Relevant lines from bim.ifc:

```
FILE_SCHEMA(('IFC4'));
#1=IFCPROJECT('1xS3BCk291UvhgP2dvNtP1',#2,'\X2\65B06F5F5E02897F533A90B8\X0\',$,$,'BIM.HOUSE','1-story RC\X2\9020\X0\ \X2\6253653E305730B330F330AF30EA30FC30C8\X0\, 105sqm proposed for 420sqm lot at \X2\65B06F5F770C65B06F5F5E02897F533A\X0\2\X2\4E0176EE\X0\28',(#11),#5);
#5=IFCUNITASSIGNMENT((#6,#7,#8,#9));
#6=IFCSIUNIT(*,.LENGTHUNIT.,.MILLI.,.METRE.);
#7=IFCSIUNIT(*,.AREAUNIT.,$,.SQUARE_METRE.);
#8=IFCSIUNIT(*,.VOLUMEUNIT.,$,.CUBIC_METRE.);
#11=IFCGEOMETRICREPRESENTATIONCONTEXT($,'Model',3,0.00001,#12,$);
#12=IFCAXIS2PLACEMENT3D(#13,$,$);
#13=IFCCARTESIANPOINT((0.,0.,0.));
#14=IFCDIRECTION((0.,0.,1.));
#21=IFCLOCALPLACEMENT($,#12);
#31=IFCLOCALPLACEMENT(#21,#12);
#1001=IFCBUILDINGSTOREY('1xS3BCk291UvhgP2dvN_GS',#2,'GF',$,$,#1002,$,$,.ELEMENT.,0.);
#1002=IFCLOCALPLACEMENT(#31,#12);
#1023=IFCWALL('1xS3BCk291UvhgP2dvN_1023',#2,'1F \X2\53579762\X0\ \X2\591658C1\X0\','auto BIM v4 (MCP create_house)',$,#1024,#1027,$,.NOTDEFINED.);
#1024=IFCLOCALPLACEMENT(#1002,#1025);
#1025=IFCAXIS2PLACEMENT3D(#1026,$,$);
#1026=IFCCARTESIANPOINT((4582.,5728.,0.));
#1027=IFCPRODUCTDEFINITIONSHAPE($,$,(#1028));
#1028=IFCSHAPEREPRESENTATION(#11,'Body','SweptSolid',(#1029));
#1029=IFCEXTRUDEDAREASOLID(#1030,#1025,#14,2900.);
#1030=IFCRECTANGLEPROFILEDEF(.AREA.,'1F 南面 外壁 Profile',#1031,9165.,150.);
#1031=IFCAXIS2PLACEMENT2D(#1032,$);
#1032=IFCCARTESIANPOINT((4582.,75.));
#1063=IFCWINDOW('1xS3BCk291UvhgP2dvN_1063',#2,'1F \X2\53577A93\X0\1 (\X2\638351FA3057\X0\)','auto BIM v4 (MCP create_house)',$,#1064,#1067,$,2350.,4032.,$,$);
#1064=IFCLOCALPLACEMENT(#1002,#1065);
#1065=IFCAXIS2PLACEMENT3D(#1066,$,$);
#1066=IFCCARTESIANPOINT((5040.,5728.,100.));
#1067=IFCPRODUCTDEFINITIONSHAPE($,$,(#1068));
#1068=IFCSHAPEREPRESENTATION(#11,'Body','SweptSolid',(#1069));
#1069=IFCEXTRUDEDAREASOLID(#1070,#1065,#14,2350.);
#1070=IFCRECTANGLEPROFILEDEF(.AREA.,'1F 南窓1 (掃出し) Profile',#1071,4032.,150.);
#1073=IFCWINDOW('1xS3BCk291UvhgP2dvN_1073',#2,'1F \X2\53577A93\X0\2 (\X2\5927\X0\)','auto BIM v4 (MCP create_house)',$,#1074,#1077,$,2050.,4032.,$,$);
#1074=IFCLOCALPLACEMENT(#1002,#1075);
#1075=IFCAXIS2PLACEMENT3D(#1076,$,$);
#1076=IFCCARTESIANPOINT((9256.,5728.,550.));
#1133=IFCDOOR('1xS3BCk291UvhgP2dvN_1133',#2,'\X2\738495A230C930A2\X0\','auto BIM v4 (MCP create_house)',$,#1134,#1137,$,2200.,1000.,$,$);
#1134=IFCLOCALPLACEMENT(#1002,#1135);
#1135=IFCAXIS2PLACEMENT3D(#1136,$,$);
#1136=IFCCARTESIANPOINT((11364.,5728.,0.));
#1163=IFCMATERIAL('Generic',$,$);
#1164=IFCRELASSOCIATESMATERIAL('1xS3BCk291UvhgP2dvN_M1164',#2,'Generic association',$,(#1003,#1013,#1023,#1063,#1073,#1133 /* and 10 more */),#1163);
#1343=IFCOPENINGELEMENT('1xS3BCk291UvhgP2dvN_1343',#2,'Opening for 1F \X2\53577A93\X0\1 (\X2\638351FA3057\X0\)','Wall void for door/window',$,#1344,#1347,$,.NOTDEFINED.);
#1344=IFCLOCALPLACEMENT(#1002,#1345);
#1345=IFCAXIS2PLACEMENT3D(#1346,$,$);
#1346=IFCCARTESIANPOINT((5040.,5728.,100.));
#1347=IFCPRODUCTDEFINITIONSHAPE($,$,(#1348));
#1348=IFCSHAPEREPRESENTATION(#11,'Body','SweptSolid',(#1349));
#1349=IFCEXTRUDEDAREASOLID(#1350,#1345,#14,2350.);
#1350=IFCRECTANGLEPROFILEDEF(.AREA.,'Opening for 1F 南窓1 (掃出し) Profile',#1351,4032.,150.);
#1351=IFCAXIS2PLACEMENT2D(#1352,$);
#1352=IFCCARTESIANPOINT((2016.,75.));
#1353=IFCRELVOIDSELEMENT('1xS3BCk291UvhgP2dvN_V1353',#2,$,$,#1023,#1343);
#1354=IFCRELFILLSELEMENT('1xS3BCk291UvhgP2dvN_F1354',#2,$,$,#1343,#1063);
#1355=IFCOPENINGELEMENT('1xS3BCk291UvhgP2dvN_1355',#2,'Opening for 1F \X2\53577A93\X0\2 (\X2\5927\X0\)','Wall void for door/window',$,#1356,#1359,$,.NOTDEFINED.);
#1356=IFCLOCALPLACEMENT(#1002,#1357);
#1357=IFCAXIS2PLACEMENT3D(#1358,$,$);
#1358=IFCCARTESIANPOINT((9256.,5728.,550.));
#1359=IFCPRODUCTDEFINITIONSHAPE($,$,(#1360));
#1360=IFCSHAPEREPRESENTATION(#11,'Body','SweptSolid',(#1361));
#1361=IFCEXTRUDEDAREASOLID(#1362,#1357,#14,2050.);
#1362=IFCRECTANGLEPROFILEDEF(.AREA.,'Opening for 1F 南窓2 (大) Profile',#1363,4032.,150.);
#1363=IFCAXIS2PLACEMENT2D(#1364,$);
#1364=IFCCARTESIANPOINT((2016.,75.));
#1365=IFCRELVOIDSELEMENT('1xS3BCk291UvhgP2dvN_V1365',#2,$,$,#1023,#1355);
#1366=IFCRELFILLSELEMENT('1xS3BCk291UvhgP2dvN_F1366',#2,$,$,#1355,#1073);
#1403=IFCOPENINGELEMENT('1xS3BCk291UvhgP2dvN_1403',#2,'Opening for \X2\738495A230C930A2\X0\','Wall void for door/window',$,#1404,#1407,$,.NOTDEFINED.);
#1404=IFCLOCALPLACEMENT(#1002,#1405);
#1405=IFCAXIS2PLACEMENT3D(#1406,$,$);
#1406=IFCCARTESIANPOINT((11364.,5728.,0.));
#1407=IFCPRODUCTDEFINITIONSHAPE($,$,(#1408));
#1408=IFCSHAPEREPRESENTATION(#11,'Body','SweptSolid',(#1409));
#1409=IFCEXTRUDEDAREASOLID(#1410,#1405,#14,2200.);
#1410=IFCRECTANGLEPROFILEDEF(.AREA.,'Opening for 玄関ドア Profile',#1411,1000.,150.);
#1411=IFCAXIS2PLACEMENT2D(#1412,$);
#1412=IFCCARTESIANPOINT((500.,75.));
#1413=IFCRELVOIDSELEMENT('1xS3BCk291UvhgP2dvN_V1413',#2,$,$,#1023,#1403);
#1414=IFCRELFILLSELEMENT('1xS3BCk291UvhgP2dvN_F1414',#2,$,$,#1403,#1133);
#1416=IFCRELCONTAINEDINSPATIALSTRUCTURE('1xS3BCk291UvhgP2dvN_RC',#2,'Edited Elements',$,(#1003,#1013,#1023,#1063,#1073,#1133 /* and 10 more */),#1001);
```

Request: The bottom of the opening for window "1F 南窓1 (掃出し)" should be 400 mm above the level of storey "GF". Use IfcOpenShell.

```python
import numpy as np
import ifcopenshell
import ifcopenshell.api.geometry
import ifcopenshell.geom
import ifcopenshell.util.element
import ifcopenshell.util.placement
import ifcopenshell.util.shape
import ifcopenshell.util.unit

model = ifcopenshell.open("bim.ifc")
unit_scale = ifcopenshell.util.unit.calculate_unit_scale(model)

window = model.by_id(1063)
opening = window.FillsVoids[0].RelatingOpeningElement
storey = ifcopenshell.util.element.get_container(window, ifc_class="IfcBuildingStorey")
level = ifcopenshell.util.placement.get_local_placement(storey.ObjectPlacement)[2, 3]

# The opening's origin need not be at the sill, so measure its lowest point.
shape = ifcopenshell.geom.create_shape(ifcopenshell.geom.settings(), opening)
bottom = ifcopenshell.util.shape.get_shape_bottom_elevation(shape, shape.geometry) / unit_scale
dz = level + 400.0 - bottom

shift = np.array([0.0, 0.0, dz])
# The window is not placed relative to its opening, so move both.
for product in (opening, window):
    matrix = ifcopenshell.util.placement.get_local_placement(product.ObjectPlacement)
    matrix[:3, 3] += shift
    ifcopenshell.api.geometry.edit_object_placement(model, product=product, matrix=matrix, is_si=False)

print(f"moved by {dz * unit_scale:+.3f} m")

model.write("bim_rev.ifc")
```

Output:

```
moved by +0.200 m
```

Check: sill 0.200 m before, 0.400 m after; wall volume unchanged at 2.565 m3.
